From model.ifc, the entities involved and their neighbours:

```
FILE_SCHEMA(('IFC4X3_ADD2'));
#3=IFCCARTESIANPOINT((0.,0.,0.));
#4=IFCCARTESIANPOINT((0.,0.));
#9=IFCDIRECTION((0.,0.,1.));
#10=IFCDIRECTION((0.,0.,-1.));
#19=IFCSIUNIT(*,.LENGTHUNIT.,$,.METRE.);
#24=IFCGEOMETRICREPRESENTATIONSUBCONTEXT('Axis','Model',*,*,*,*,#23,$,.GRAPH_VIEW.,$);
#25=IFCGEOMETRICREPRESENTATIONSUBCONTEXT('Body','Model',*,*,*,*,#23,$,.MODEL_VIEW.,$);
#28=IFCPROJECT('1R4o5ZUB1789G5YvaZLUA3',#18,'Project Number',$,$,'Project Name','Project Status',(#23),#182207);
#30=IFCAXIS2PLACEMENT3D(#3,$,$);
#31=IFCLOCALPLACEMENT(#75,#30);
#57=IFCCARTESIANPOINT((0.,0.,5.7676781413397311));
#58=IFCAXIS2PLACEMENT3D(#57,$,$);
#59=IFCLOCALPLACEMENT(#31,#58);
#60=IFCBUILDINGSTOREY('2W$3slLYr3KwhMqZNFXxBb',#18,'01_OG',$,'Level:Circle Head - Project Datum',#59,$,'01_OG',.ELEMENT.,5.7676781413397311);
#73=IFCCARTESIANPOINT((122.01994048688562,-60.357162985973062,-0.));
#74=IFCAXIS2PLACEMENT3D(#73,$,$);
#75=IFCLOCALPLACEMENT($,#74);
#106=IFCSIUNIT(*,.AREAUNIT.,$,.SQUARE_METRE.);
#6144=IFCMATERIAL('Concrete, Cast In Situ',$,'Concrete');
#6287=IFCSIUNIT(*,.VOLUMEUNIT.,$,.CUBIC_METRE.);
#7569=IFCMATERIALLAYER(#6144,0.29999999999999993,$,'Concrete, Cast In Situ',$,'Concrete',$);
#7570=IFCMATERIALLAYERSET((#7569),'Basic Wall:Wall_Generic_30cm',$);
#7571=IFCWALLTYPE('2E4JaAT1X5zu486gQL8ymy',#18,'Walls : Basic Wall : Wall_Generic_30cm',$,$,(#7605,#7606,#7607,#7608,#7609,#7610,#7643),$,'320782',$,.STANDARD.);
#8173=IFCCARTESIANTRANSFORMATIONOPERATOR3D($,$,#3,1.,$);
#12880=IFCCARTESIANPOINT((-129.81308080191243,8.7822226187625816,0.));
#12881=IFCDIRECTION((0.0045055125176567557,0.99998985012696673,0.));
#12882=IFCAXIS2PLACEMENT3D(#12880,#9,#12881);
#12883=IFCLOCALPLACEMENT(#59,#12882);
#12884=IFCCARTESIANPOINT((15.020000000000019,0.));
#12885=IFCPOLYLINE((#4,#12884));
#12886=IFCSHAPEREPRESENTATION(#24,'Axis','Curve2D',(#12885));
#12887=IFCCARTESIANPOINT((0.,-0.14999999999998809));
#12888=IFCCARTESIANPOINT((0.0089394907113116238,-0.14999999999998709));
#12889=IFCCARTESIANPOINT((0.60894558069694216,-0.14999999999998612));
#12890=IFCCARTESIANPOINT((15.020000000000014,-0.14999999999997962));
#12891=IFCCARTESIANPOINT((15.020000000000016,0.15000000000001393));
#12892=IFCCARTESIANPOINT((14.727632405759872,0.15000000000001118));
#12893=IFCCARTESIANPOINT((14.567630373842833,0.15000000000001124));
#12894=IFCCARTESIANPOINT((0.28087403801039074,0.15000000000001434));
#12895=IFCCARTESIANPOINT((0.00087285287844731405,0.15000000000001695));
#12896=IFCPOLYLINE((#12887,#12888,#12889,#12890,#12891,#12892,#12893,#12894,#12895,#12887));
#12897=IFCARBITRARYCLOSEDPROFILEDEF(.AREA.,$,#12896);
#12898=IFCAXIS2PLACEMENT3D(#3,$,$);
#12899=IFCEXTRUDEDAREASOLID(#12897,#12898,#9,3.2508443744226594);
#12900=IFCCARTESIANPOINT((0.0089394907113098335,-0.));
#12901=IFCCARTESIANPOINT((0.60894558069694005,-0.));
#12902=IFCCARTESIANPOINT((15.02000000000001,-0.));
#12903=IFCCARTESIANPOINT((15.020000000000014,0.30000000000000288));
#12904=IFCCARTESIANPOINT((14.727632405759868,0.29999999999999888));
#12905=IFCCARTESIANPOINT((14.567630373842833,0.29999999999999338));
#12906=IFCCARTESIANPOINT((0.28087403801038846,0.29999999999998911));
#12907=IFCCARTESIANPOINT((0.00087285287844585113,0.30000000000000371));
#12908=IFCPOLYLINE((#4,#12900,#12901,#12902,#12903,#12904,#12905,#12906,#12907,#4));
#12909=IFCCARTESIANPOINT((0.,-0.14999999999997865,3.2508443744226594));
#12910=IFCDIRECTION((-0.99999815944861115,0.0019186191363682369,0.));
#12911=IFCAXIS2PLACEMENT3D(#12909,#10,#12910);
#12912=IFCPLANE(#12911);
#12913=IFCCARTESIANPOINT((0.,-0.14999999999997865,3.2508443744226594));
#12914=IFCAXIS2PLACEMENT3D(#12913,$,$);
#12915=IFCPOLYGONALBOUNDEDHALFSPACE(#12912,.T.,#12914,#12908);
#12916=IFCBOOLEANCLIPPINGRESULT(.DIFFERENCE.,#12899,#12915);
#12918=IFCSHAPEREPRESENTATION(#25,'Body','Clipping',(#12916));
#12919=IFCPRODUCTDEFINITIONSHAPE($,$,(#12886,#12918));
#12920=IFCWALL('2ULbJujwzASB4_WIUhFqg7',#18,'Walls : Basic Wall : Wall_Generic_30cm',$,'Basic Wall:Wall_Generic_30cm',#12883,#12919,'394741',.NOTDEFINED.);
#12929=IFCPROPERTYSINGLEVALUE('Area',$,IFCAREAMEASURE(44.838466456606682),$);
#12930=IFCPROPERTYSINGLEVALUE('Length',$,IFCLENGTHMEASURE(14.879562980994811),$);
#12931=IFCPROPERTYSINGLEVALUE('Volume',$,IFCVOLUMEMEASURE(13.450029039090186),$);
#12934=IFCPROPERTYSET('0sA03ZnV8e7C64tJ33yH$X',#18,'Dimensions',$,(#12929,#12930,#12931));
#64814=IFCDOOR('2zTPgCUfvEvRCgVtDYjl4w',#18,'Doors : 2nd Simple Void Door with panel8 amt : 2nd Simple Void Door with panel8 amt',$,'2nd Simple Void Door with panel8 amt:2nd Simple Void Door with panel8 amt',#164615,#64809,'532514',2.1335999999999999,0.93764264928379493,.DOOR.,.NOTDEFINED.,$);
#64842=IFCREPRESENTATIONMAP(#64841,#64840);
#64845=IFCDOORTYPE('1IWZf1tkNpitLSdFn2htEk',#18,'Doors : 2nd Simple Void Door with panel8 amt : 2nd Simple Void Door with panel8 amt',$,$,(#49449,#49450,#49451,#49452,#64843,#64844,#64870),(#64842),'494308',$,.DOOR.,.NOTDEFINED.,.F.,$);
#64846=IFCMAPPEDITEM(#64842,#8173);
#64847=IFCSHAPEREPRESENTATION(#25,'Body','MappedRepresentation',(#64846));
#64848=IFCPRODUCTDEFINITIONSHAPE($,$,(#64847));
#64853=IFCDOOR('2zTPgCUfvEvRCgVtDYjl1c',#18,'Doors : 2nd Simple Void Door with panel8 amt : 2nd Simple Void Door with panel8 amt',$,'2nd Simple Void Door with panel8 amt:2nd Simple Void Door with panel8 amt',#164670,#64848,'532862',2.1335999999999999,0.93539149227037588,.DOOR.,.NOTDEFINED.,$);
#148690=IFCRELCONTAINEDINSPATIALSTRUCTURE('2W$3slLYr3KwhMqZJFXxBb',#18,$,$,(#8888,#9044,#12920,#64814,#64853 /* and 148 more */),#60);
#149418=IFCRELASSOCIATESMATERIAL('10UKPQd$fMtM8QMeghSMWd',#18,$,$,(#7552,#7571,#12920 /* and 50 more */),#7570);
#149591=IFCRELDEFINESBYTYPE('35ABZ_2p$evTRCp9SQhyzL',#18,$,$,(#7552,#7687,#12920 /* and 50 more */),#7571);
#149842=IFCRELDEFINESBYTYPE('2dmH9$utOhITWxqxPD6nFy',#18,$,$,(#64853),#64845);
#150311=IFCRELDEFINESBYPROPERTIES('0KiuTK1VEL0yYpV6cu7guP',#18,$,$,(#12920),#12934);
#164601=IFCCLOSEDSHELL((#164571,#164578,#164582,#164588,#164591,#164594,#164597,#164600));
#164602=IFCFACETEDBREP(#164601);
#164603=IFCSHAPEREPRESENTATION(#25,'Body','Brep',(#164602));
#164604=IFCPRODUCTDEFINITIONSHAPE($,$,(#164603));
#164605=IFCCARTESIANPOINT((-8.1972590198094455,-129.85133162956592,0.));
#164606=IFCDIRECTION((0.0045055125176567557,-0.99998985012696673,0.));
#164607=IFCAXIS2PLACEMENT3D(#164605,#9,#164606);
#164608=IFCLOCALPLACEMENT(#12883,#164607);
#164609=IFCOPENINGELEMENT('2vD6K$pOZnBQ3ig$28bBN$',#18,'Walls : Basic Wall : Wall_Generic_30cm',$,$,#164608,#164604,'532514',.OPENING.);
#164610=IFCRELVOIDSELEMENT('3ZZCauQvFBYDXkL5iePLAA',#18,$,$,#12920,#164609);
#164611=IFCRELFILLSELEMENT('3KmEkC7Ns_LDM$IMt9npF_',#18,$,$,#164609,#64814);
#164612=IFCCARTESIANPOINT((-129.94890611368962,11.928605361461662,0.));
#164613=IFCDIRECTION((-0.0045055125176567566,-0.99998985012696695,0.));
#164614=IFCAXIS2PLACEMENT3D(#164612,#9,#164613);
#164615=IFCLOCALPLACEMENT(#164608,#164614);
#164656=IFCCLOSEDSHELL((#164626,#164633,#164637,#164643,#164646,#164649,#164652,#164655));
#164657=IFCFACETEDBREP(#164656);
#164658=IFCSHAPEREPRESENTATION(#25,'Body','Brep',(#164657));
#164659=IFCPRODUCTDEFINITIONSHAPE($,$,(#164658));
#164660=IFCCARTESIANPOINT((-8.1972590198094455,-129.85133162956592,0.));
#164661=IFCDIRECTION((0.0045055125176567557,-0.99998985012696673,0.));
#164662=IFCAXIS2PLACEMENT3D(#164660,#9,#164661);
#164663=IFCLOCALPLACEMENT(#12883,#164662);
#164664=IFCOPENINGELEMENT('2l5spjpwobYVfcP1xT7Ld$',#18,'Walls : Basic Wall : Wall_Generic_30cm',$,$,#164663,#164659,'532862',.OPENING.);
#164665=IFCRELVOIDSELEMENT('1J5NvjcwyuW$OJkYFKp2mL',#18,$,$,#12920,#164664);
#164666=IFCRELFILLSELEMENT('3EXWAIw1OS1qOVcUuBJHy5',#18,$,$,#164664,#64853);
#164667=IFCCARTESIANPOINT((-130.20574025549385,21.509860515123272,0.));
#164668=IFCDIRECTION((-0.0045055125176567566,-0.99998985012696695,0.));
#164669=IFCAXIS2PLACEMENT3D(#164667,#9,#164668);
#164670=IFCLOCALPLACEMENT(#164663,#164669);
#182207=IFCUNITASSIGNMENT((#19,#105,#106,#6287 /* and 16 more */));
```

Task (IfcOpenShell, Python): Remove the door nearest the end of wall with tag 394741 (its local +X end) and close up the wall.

```python
import ifcopenshell
import ifcopenshell.api.feature
import ifcopenshell.api.pset
import ifcopenshell.api.root
import ifcopenshell.geom
import ifcopenshell.util.element
import ifcopenshell.util.shape
import ifcopenshell.util.unit

model = ifcopenshell.open("model.ifc")
area_scale = ifcopenshell.util.unit.calculate_unit_scale(model, "AREAUNIT")
volume_scale = ifcopenshell.util.unit.calculate_unit_scale(model, "VOLUMEUNIT")
settings = ifcopenshell.geom.settings()


def volume(element):
    """Net volume in cubic metres, openings subtracted."""
    shape = ifcopenshell.geom.create_shape(settings, element)
    return ifcopenshell.util.shape.get_volume(shape.geometry)


door = model.by_id(64853)
opening = door.FillsVoids[0].RelatingOpeningElement
wall = opening.VoidsElements[0].RelatingBuildingElement
before = volume(wall)

ifcopenshell.api.root.remove_product(model, product=door)
ifcopenshell.api.feature.remove_feature(model, feature=opening)

after = volume(wall)
thickness = 0.3  # wall thickness in metres

# Update the wall's stored quantities.
pset = model.by_id(ifcopenshell.util.element.get_pset(wall, "Dimensions", should_inherit=False)["id"])
ifcopenshell.api.pset.edit_pset(model, pset=pset, properties={
    "Area": model.create_entity("IfcAreaMeasure", after / thickness / area_scale),
    "Volume": model.create_entity("IfcVolumeMeasure", after / volume_scale),
})

print(f"wall volume {before:.3f} -> {after:.3f} m3")

model.write("model_updated.ifc")
```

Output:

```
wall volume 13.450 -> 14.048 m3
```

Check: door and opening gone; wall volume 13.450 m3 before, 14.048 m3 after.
